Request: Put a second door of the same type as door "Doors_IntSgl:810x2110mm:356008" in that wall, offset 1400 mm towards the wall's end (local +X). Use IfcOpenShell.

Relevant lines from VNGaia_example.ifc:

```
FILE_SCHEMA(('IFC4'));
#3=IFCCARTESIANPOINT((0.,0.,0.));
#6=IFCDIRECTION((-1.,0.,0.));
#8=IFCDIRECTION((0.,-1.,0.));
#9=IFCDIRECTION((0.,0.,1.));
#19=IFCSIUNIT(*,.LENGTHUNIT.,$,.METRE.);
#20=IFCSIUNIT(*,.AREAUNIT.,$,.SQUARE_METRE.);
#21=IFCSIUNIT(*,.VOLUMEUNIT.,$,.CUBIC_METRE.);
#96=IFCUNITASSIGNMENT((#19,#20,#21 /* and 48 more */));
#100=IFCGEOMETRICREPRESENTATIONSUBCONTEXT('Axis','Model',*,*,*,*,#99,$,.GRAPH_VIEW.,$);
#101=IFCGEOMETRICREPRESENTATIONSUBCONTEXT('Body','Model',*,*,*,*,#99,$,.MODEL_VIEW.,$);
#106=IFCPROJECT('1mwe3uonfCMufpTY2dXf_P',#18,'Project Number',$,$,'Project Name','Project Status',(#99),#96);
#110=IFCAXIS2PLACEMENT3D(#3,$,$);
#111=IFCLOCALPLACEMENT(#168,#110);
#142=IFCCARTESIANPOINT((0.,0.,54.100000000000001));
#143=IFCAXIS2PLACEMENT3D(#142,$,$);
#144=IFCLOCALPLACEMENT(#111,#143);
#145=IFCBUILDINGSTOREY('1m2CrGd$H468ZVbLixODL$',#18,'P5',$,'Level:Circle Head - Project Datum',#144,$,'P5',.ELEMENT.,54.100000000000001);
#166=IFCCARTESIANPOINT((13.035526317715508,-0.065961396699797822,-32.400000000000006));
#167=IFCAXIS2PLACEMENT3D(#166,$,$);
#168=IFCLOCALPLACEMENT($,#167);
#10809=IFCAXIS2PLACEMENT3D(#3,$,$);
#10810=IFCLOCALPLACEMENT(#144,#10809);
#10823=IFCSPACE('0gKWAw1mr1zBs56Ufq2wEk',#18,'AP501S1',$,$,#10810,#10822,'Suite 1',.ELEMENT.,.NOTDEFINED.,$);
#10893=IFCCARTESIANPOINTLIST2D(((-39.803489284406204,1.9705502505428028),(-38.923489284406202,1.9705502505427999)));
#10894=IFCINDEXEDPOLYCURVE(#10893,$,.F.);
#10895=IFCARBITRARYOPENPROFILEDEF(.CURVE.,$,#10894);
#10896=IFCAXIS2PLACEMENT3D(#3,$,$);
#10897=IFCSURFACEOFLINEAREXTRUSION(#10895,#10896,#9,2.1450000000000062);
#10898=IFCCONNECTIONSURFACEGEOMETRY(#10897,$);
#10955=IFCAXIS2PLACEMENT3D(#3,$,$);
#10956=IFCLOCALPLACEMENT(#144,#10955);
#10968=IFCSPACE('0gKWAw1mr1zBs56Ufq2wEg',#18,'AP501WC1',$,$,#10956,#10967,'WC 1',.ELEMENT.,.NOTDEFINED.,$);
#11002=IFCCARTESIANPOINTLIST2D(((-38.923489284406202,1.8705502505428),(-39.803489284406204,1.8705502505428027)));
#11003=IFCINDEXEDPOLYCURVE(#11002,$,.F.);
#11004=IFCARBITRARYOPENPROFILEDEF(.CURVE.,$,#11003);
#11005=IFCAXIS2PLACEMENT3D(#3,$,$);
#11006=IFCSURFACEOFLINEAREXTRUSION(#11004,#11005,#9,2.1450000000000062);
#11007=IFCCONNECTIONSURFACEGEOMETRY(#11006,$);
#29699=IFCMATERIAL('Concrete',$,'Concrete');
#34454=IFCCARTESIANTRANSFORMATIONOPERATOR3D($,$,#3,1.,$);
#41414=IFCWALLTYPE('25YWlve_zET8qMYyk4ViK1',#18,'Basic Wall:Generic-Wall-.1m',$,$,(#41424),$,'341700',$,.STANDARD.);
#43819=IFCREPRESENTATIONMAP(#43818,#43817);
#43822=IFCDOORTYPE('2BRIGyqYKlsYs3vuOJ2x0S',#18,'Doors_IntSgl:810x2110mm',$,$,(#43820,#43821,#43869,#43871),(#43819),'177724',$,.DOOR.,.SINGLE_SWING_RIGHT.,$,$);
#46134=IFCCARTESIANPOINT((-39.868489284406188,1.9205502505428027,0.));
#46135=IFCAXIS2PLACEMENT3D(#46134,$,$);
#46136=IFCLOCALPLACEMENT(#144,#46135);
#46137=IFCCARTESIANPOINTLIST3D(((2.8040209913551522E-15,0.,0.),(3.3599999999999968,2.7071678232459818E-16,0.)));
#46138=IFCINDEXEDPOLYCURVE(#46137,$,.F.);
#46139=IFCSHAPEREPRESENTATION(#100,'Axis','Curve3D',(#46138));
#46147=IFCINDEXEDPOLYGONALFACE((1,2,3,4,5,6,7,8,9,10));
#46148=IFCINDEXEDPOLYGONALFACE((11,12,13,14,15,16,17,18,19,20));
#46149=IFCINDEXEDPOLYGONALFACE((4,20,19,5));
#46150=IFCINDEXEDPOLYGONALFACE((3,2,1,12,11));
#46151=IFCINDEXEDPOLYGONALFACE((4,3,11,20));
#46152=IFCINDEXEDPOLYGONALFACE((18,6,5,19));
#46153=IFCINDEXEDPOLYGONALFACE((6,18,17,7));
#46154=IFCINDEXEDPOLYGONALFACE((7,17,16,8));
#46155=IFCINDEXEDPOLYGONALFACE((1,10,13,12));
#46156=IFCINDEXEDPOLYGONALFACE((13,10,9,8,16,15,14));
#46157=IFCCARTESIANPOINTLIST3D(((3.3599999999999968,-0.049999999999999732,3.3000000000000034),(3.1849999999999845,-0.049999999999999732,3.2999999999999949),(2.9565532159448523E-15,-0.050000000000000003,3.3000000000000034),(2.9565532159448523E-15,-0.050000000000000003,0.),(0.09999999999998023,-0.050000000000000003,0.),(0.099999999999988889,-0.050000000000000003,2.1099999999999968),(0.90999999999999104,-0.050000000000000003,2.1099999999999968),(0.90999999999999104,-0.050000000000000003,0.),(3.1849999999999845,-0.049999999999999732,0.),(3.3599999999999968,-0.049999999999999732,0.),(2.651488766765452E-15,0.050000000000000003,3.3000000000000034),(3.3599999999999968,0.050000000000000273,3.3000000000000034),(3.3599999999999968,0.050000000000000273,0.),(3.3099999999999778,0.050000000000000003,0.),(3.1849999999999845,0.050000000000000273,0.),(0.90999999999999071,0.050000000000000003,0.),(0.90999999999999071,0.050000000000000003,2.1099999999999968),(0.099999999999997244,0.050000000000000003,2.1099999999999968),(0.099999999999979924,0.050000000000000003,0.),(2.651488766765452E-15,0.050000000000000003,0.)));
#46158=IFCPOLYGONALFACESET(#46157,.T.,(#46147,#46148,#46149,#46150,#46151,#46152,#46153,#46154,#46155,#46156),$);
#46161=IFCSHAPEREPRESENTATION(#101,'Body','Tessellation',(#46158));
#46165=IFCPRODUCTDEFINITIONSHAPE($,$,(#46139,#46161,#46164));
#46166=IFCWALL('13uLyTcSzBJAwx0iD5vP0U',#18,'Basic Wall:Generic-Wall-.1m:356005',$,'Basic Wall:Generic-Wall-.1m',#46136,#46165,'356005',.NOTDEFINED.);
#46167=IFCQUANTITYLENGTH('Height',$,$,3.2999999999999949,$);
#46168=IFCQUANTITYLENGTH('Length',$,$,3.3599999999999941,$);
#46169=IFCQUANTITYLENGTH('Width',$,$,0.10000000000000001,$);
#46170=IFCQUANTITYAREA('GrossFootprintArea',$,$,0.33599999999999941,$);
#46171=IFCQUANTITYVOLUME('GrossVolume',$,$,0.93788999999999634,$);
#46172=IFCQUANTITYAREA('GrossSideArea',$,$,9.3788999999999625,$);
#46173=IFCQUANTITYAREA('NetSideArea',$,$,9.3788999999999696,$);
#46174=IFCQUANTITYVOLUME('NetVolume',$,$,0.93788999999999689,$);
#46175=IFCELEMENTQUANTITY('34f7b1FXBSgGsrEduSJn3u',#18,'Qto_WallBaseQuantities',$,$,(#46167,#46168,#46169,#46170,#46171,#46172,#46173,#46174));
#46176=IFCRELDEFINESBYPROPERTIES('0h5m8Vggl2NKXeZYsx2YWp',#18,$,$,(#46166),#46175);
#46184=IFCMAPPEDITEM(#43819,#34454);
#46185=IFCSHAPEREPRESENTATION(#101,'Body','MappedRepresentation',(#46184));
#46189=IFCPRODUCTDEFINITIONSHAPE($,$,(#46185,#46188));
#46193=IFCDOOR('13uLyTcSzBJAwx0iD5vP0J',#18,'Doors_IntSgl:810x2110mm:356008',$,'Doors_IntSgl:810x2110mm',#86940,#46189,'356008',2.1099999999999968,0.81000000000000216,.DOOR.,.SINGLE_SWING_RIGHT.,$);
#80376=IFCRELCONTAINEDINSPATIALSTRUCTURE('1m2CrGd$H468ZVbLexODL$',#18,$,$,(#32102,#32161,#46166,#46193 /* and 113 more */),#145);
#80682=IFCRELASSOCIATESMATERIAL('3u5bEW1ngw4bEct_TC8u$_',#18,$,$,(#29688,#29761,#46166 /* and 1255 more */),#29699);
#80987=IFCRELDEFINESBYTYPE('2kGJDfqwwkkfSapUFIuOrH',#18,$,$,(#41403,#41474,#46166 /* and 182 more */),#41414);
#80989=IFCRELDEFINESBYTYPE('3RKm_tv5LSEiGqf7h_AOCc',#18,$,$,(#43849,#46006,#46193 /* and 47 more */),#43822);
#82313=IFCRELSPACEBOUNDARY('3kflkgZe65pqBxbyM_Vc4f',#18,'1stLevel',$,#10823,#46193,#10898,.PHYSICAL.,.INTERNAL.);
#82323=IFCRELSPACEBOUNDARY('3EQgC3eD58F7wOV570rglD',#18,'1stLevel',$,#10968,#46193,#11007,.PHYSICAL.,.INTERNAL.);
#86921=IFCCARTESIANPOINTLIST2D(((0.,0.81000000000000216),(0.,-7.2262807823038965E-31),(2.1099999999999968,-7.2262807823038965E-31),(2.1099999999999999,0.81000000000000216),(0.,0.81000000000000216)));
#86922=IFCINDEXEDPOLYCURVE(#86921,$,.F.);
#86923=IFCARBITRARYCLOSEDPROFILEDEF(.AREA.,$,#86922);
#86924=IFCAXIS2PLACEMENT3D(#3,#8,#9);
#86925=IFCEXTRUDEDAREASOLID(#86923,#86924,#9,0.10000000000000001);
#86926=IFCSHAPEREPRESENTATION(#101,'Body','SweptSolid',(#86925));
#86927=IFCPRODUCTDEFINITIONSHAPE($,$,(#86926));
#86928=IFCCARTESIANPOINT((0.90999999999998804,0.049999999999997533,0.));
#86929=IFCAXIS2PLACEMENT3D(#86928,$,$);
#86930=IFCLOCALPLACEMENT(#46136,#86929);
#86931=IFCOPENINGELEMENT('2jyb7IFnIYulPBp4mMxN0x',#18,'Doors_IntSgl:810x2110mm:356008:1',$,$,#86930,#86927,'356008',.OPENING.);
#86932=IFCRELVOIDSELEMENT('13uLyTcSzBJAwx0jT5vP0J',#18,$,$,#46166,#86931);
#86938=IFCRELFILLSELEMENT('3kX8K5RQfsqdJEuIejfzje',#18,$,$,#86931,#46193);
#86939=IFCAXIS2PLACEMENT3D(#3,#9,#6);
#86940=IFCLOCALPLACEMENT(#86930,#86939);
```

```python
import numpy as np
import ifcopenshell
import ifcopenshell.api.feature
import ifcopenshell.api.geometry
import ifcopenshell.api.pset
import ifcopenshell.api.root
import ifcopenshell.geom
import ifcopenshell.util.element
import ifcopenshell.util.placement
import ifcopenshell.util.shape
import ifcopenshell.util.unit

model = ifcopenshell.open("VNGaia_example.ifc")
area_scale = ifcopenshell.util.unit.calculate_unit_scale(model, "AREAUNIT")
volume_scale = ifcopenshell.util.unit.calculate_unit_scale(model, "VOLUMEUNIT")
settings = ifcopenshell.geom.settings()


def volume(element):
    """Net volume in cubic metres, openings subtracted."""
    shape = ifcopenshell.geom.create_shape(settings, element)
    return ifcopenshell.util.shape.get_volume(shape.geometry)


def reuse_history(source, copy):
    """copy_class also copies each property set's owner history, people and application; keep the originals."""
    for rel in copy.IsDefinedBy:
        if rel.is_a("IfcRelDefinesByProperties") and (history := rel.RelatingPropertyDefinition.OwnerHistory):
            rel.RelatingPropertyDefinition.OwnerHistory = source.OwnerHistory
            ifcopenshell.util.element.remove_deep2(model, history)


door = model.by_guid("13uLyTcSzBJAwx0iD5vP0J")
opening = door.FillsVoids[0].RelatingOpeningElement
wall = opening.VoidsElements[0].RelatingBuildingElement
before = volume(wall)
shift = ifcopenshell.util.placement.get_local_placement(wall.ObjectPlacement)[:3, 0] * 1.4

# copy_class copies the void relationship, type, container and properties, but no geometry.
new_opening = ifcopenshell.api.root.copy_class(model, product=opening)
new_opening.Representation = ifcopenshell.util.element.copy_deep(
    model, opening.Representation, exclude=["IfcGeometricRepresentationContext", "IfcRepresentationMap"]
)
new_opening.Name = "Doors_IntSgl:810x2110mm"
new_opening.Tag = None
reuse_history(opening, new_opening)
new_door = ifcopenshell.api.root.copy_class(model, product=door)
new_door.Representation = ifcopenshell.util.element.copy_deep(
    model, door.Representation, exclude=["IfcGeometricRepresentationContext", "IfcRepresentationMap"]
)
new_door.Name = "Doors_IntSgl:810x2110mm"
new_door.Tag = None
reuse_history(door, new_door)
ifcopenshell.api.feature.add_filling(model, opening=new_opening, element=new_door)

for old, new in ((opening, new_opening), (door, new_door)):
    matrix = ifcopenshell.util.placement.get_local_placement(old.ObjectPlacement)
    matrix[:3, 3] += shift
    ifcopenshell.api.geometry.edit_object_placement(model, product=new, matrix=matrix, is_si=False)

# The copied space boundaries still share their surfaces with the original.
for rel in new_door.ProvidesBoundaries:
    if rel.ConnectionGeometry:
        rel.ConnectionGeometry = ifcopenshell.util.element.copy_deep(model, rel.ConnectionGeometry)

# Space boundary surfaces are stored in each space's coordinates; move them too.
for rel in new_door.ProvidesBoundaries:
    if not rel.ConnectionGeometry:
        continue
    surface = rel.ConnectionGeometry.SurfaceOnRelatingElement
    space_matrix = ifcopenshell.util.placement.get_local_placement(rel.RelatingSpace.ObjectPlacement)
    point = np.array(surface.Position.Location.Coordinates) + space_matrix[:3, :3].T @ shift
    surface.Position = model.createIfcAxis2Placement3D(
        model.createIfcCartesianPoint(point.tolist()), surface.Position.Axis, surface.Position.RefDirection
    )

after = volume(wall)
thickness = 0.1  # wall thickness in metres

# Update the wall's stored quantities.
qto = model.by_id(ifcopenshell.util.element.get_pset(wall, "Qto_WallBaseQuantities", should_inherit=False)["id"])
ifcopenshell.api.pset.edit_qto(model, qto=qto, properties={
    "NetSideArea": after / thickness / area_scale,
    "NetVolume": after / volume_scale,
})

print(f"wall volume {before:.3f} -> {after:.3f} m3")

model.write("VNGaia_example_updated.ifc")
```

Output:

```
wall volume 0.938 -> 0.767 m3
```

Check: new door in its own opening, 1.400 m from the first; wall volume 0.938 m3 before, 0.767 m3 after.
